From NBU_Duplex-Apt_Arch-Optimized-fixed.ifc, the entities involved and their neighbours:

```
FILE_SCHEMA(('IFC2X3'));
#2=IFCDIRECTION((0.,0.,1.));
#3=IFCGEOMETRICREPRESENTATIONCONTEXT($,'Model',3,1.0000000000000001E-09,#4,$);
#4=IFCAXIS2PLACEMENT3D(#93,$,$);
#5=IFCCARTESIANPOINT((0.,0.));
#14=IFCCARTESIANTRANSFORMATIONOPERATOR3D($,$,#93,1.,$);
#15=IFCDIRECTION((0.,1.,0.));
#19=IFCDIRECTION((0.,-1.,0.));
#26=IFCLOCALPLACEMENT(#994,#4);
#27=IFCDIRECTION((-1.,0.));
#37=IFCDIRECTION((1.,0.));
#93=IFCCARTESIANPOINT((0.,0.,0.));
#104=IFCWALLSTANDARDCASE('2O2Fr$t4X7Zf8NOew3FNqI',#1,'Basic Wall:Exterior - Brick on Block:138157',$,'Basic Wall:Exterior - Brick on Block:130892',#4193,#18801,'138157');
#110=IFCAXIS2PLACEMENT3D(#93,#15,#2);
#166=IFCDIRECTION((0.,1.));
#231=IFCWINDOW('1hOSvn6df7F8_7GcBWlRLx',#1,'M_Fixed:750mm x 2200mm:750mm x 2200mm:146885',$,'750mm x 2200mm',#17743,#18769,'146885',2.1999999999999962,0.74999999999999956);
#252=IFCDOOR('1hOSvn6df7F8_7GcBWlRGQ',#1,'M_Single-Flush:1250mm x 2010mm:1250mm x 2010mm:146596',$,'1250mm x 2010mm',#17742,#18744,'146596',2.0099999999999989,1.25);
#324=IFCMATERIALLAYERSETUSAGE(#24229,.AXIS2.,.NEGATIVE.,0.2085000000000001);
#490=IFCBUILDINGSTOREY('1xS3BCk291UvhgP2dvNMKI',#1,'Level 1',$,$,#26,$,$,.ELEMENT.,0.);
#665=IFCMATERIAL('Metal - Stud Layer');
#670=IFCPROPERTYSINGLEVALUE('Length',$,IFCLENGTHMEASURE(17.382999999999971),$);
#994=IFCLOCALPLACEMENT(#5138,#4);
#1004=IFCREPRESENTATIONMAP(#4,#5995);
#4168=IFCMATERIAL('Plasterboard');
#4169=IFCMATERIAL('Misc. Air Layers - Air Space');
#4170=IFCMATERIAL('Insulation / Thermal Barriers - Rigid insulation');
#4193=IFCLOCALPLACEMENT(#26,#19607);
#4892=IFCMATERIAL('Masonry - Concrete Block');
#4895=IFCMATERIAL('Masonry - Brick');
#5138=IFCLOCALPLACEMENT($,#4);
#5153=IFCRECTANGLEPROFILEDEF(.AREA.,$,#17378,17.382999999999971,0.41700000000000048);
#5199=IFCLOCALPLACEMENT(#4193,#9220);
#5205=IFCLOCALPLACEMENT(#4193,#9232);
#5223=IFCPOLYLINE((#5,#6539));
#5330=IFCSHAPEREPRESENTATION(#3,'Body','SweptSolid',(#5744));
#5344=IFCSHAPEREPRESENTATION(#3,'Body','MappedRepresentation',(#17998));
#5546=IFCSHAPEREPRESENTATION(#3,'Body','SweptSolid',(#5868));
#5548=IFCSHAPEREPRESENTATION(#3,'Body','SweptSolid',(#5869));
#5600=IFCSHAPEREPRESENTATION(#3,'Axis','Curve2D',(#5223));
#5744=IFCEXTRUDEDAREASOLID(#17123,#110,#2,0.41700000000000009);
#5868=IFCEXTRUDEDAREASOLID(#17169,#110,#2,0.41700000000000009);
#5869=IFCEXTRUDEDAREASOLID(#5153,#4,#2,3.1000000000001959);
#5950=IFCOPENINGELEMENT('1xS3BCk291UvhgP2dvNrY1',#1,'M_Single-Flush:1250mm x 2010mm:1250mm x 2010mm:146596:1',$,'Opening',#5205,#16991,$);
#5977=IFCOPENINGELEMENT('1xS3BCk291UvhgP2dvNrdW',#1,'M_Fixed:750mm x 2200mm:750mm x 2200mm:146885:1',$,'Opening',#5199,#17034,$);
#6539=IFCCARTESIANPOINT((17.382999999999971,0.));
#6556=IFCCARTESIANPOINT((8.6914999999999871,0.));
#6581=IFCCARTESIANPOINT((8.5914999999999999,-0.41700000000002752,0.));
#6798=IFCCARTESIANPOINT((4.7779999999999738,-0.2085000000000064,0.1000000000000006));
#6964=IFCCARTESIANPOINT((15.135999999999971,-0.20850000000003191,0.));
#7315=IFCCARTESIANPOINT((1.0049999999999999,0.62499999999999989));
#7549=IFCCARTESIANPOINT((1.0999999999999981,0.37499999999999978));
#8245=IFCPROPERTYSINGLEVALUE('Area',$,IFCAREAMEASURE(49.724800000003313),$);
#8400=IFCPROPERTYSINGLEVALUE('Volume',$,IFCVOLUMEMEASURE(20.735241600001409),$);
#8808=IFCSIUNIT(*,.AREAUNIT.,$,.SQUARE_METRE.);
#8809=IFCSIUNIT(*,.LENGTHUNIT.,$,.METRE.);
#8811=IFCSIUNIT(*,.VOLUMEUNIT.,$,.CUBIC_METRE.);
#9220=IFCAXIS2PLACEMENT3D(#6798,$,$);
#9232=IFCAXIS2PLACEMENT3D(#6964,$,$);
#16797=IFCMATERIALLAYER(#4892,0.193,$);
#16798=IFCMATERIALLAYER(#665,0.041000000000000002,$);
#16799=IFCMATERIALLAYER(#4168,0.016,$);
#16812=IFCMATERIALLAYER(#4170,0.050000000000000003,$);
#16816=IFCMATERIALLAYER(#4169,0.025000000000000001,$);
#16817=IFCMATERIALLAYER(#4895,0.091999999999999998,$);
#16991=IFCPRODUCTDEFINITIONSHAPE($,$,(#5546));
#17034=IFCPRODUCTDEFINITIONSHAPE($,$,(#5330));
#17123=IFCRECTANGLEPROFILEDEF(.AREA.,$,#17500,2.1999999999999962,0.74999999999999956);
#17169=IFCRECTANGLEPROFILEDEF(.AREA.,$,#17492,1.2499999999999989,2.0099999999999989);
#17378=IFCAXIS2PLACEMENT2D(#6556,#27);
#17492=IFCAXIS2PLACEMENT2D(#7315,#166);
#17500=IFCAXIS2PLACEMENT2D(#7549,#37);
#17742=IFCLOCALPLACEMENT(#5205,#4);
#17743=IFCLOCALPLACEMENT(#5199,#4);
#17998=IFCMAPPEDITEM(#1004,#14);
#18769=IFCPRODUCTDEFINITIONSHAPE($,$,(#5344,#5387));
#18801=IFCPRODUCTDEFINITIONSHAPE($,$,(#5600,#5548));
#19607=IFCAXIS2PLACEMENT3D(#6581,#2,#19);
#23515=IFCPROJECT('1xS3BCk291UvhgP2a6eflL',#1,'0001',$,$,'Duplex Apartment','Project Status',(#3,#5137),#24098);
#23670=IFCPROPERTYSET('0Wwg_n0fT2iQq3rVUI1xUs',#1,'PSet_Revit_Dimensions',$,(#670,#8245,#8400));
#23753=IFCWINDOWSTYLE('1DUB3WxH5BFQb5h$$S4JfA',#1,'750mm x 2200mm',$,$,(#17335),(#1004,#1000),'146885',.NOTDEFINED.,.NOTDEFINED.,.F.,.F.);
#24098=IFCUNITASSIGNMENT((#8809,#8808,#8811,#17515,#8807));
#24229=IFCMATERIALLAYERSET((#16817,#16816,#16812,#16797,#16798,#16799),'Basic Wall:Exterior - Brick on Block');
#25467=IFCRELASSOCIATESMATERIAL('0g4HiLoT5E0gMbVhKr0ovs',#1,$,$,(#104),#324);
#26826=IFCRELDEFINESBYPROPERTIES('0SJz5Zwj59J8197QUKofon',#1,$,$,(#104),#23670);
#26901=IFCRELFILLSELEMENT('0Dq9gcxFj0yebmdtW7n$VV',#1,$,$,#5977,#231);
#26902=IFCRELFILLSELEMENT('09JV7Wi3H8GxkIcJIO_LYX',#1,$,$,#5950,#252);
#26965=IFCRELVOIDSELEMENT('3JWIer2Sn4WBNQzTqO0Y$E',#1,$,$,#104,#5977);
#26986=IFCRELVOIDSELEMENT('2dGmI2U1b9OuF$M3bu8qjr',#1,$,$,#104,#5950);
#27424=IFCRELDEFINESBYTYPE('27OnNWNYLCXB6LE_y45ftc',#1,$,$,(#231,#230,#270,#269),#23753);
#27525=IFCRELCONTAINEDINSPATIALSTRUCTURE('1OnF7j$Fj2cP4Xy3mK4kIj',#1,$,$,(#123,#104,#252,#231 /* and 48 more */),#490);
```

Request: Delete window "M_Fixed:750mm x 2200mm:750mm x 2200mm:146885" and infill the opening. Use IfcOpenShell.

```python
import ifcopenshell
import ifcopenshell.api.feature
import ifcopenshell.api.pset
import ifcopenshell.api.root
import ifcopenshell.geom
import ifcopenshell.util.element
import ifcopenshell.util.shape
import ifcopenshell.util.unit

model = ifcopenshell.open("NBU_Duplex-Apt_Arch-Optimized-fixed.ifc")
area_scale = ifcopenshell.util.unit.calculate_unit_scale(model, "AREAUNIT")
volume_scale = ifcopenshell.util.unit.calculate_unit_scale(model, "VOLUMEUNIT")
settings = ifcopenshell.geom.settings()


def volume(element):
    """Net volume in cubic metres, openings subtracted."""
    shape = ifcopenshell.geom.create_shape(settings, element)
    return ifcopenshell.util.shape.get_volume(shape.geometry)


window = model.by_id(231)
opening = window.FillsVoids[0].RelatingOpeningElement
wall = opening.VoidsElements[0].RelatingBuildingElement
before = volume(wall)

ifcopenshell.api.root.remove_product(model, product=window)
ifcopenshell.api.feature.remove_feature(model, feature=opening)

after = volume(wall)
thickness = 0.417  # wall thickness in metres

# Update the wall's stored quantities.
pset = model.by_id(ifcopenshell.util.element.get_pset(wall, "PSet_Revit_Dimensions", should_inherit=False)["id"])
ifcopenshell.api.pset.edit_pset(model, pset=pset, properties={
    "Area": model.create_entity("IfcAreaMeasure", after / thickness / area_scale),
    "Volume": model.create_entity("IfcVolumeMeasure", after / volume_scale),
})

print(f"wall volume {before:.3f} -> {after:.3f} m3")

model.write("NBU_Duplex-Apt_Arch-Optimized-fixed_rev.ifc")
```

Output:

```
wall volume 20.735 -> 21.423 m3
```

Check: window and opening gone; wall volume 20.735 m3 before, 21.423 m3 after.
